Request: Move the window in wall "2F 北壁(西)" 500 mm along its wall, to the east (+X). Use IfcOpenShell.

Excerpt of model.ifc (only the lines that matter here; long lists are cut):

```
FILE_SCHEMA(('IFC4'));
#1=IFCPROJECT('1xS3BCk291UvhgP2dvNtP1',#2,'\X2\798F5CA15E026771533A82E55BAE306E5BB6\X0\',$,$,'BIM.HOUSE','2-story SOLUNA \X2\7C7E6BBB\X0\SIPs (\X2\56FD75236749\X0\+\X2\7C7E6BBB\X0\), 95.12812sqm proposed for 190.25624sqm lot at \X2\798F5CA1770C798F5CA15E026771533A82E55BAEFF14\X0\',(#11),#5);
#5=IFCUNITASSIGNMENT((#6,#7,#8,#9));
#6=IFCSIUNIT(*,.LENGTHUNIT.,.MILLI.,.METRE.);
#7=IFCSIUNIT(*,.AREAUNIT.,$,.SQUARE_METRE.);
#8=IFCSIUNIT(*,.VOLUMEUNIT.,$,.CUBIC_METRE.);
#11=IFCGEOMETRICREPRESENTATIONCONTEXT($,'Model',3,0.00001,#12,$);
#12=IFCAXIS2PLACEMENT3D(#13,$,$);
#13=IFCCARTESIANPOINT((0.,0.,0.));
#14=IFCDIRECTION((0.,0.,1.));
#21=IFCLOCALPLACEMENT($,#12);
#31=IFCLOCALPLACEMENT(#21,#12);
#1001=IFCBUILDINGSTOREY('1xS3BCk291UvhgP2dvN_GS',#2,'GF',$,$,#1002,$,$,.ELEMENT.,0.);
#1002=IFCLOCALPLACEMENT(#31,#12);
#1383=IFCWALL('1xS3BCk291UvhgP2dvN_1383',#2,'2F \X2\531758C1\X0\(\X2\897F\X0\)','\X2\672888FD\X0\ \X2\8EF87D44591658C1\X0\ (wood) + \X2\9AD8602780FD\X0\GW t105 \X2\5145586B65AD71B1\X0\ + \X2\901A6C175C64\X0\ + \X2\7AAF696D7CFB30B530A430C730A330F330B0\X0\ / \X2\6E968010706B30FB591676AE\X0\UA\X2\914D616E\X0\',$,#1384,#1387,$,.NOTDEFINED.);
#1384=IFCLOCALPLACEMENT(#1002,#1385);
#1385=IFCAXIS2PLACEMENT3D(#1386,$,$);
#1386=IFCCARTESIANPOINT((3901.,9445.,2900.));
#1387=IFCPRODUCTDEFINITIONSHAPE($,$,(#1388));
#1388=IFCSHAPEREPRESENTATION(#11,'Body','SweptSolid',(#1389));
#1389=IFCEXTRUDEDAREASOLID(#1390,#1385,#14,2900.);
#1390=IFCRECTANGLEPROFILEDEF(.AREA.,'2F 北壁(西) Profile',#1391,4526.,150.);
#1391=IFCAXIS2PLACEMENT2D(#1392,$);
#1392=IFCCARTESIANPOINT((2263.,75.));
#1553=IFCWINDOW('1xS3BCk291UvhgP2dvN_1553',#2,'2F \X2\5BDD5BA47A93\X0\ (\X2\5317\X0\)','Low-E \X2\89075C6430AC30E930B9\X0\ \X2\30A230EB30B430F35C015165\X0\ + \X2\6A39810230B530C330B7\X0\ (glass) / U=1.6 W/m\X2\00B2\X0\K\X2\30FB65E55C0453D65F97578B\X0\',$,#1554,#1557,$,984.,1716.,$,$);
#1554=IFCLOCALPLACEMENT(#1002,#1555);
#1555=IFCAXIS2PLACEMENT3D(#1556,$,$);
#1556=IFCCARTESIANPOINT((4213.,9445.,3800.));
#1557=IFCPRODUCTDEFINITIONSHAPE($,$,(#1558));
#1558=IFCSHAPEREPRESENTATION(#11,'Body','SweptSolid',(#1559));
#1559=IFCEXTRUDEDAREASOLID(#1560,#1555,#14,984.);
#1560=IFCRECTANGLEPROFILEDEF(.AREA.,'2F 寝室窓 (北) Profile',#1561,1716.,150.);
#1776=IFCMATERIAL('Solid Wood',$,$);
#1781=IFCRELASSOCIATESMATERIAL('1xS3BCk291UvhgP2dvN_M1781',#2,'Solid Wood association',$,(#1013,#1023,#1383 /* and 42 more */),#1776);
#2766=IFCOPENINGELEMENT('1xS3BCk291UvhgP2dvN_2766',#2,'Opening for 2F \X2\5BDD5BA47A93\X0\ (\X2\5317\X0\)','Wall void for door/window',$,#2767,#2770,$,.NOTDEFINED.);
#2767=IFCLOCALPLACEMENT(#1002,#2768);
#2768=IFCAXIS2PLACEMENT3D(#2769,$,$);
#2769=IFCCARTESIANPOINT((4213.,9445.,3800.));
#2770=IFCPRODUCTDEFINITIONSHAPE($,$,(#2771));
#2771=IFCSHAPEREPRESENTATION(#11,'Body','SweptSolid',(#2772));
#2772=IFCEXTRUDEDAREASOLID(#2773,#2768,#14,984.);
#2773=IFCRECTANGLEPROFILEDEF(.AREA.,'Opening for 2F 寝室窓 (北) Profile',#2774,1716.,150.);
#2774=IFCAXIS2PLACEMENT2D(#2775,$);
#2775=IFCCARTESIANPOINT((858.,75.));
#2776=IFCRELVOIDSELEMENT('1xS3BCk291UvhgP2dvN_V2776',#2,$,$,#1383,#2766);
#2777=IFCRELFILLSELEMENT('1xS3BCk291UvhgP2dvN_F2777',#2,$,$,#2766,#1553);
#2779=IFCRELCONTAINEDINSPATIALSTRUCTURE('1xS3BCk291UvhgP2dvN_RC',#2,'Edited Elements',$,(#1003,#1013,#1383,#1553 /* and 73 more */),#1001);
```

```python
import ifcopenshell
import ifcopenshell.api.geometry
import ifcopenshell.util.placement

model = ifcopenshell.open("model.ifc")

window = model.by_guid("1xS3BCk291UvhgP2dvN_1553")
opening = window.FillsVoids[0].RelatingOpeningElement
wall = opening.VoidsElements[0].RelatingBuildingElement

wall_matrix = ifcopenshell.util.placement.get_local_placement(wall.ObjectPlacement)
shift = wall_matrix[:3, 0] * 500.0
before = ifcopenshell.util.placement.get_local_placement(window.ObjectPlacement)[:3, 3].copy()

# The window is not placed relative to its opening, so move both.
for product in (opening, window):
    matrix = ifcopenshell.util.placement.get_local_placement(product.ObjectPlacement)
    matrix[:3, 3] += shift
    ifcopenshell.api.geometry.edit_object_placement(model, product=product, matrix=matrix, is_si=False)

after = ifcopenshell.util.placement.get_local_placement(window.ObjectPlacement)[:3, 3]
print("window moved by", (after - before).round(3) + 0.0)

model.write("model_rev.ifc")
```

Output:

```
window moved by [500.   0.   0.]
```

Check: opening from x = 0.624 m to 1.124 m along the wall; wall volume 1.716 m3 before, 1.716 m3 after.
